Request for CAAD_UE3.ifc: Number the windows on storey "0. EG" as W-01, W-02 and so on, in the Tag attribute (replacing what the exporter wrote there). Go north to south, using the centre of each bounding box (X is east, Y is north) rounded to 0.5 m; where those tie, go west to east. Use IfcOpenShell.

First a look at what the model holds.

```python
import ifcopenshell
import ifcopenshell.util.element
import ifcopenshell.util.placement

model = ifcopenshell.open("CAAD_UE3.ifc")
print(model.schema)
storey = next(s for s in model.by_type("IfcBuildingStorey") if s.Name == "0. EG")
windows = [e for e in ifcopenshell.util.element.get_decomposition(storey) if e.is_a("IfcWindow")]
for e in sorted(windows, key=lambda e: e.id()):
    origin = ifcopenshell.util.placement.get_local_placement(e.ObjectPlacement)[:3, 3]
    print(e.id(), e.Tag, e.Name, origin.round(2) + 0.0, sep=" | ")
```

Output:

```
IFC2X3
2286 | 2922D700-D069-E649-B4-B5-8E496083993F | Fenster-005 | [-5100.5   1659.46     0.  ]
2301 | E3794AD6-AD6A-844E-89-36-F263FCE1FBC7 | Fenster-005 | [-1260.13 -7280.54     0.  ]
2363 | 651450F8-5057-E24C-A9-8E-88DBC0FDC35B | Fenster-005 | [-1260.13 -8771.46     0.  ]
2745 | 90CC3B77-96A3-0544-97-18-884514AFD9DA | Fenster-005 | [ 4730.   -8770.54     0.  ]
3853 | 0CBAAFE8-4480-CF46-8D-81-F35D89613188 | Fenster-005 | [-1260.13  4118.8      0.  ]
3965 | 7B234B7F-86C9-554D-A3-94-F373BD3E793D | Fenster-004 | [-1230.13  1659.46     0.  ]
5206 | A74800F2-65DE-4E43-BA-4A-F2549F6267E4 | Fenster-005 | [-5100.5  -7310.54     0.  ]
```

```python
import ifcopenshell
import ifcopenshell.geom
import ifcopenshell.util.element
import ifcopenshell.util.shape

model = ifcopenshell.open("CAAD_UE3.ifc")
settings = ifcopenshell.geom.settings()
settings.set("use-world-coords", True)


def centre(element):
    shape = ifcopenshell.geom.create_shape(settings, element)
    return ifcopenshell.util.shape.get_bbox_centroid(shape.geometry)


storey = next(s for s in model.by_type("IfcBuildingStorey") if s.Name == "0. EG")
windows = [e for e in ifcopenshell.util.element.get_decomposition(storey) if e.is_a("IfcWindow")]

# Insertion points can sit at a corner or the storey origin, so sort by the geometry (in metres).
centres = {e: centre(e) for e in windows}
windows.sort(key=lambda e: (-round(centres[e][1] / 0.5), centres[e][0]))

for i, e in enumerate(windows, start=1):
    number = f"W-{i:02d}"
    e.Tag = number
    print(e.id(), number)

model.write("CAAD_UE3_edited.ifc")
```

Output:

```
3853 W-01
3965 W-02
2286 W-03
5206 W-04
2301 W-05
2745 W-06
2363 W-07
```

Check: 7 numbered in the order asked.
